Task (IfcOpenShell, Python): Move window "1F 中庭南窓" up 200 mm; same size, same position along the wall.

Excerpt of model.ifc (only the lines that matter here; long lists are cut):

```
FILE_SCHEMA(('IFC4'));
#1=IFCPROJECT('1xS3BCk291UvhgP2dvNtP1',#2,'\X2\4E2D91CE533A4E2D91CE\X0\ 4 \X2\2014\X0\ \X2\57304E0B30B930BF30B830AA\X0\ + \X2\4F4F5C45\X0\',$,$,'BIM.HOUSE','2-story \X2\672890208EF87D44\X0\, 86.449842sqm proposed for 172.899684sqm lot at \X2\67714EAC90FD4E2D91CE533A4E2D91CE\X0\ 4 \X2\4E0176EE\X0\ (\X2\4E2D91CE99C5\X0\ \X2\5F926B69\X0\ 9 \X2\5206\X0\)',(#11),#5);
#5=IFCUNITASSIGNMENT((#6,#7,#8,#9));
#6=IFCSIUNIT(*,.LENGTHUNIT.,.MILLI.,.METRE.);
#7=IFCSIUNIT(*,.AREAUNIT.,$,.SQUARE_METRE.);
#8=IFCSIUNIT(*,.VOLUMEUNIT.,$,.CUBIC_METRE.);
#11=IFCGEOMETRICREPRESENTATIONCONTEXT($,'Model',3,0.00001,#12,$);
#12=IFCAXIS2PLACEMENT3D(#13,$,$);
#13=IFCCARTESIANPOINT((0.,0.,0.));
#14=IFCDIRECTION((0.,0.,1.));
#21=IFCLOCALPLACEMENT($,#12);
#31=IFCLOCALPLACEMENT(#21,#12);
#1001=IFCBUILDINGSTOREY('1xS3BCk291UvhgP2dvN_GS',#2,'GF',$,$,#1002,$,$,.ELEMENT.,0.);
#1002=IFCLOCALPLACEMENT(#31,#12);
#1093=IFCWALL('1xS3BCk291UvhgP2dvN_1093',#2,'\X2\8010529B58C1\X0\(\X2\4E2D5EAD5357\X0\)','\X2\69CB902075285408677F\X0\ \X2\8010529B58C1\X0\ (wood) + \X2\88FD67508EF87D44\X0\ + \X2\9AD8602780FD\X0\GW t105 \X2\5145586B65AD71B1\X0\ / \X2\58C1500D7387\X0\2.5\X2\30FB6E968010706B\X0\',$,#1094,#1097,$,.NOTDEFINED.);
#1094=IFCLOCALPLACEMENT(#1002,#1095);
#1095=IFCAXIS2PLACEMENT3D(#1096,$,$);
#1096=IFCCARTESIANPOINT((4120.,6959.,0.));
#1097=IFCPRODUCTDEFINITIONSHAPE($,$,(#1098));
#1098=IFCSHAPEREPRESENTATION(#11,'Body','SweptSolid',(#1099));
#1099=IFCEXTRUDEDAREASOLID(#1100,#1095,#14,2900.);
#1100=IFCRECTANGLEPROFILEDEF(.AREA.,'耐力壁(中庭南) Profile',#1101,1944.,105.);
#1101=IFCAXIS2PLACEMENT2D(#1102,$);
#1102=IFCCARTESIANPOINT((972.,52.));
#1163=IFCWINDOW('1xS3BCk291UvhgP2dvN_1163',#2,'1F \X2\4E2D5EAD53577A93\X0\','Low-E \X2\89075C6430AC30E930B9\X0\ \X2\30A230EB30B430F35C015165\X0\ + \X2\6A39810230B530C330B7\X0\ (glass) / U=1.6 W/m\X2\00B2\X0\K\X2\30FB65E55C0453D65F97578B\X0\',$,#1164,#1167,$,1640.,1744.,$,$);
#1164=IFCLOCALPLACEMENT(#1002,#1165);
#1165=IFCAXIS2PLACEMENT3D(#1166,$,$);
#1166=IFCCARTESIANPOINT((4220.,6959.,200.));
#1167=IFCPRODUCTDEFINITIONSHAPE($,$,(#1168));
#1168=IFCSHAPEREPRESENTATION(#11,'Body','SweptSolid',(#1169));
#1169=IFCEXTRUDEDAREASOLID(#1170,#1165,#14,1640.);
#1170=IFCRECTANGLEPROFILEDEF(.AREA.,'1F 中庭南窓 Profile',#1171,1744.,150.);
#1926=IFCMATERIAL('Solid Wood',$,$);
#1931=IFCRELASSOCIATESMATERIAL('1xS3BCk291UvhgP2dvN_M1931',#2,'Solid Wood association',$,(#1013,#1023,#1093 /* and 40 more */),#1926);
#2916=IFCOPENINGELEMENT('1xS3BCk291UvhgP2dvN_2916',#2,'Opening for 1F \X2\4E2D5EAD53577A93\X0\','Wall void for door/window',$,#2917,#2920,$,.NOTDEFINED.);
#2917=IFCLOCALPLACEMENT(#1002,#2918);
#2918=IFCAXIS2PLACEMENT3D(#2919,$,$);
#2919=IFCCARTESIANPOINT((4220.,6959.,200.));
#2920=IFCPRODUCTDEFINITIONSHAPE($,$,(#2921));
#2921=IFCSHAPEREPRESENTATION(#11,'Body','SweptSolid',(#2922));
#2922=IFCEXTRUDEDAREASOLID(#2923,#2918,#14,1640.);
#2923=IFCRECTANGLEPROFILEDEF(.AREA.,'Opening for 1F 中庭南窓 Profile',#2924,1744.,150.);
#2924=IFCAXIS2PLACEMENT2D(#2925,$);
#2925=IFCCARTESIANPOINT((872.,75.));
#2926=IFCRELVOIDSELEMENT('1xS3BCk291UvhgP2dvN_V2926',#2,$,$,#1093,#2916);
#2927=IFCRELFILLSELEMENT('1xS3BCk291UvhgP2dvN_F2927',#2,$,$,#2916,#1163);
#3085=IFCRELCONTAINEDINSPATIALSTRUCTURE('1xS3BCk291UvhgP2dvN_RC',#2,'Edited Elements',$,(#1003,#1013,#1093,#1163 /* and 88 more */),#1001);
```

```python
import numpy as np
import ifcopenshell
import ifcopenshell.api.geometry
import ifcopenshell.util.placement
import ifcopenshell.util.unit

model = ifcopenshell.open("model.ifc")
unit_scale = ifcopenshell.util.unit.calculate_unit_scale(model)

window = model.by_guid("1xS3BCk291UvhgP2dvN_1163")
opening = window.FillsVoids[0].RelatingOpeningElement
dz = 200.0

shift = np.array([0.0, 0.0, dz])
# The window is not placed relative to its opening, so move both.
for product in (opening, window):
    matrix = ifcopenshell.util.placement.get_local_placement(product.ObjectPlacement)
    matrix[:3, 3] += shift
    ifcopenshell.api.geometry.edit_object_placement(model, product=product, matrix=matrix, is_si=False)

print(f"moved by {dz * unit_scale:+.3f} m")

model.write("model_v2.ifc")
```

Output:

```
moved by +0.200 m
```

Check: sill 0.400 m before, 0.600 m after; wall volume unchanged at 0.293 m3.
